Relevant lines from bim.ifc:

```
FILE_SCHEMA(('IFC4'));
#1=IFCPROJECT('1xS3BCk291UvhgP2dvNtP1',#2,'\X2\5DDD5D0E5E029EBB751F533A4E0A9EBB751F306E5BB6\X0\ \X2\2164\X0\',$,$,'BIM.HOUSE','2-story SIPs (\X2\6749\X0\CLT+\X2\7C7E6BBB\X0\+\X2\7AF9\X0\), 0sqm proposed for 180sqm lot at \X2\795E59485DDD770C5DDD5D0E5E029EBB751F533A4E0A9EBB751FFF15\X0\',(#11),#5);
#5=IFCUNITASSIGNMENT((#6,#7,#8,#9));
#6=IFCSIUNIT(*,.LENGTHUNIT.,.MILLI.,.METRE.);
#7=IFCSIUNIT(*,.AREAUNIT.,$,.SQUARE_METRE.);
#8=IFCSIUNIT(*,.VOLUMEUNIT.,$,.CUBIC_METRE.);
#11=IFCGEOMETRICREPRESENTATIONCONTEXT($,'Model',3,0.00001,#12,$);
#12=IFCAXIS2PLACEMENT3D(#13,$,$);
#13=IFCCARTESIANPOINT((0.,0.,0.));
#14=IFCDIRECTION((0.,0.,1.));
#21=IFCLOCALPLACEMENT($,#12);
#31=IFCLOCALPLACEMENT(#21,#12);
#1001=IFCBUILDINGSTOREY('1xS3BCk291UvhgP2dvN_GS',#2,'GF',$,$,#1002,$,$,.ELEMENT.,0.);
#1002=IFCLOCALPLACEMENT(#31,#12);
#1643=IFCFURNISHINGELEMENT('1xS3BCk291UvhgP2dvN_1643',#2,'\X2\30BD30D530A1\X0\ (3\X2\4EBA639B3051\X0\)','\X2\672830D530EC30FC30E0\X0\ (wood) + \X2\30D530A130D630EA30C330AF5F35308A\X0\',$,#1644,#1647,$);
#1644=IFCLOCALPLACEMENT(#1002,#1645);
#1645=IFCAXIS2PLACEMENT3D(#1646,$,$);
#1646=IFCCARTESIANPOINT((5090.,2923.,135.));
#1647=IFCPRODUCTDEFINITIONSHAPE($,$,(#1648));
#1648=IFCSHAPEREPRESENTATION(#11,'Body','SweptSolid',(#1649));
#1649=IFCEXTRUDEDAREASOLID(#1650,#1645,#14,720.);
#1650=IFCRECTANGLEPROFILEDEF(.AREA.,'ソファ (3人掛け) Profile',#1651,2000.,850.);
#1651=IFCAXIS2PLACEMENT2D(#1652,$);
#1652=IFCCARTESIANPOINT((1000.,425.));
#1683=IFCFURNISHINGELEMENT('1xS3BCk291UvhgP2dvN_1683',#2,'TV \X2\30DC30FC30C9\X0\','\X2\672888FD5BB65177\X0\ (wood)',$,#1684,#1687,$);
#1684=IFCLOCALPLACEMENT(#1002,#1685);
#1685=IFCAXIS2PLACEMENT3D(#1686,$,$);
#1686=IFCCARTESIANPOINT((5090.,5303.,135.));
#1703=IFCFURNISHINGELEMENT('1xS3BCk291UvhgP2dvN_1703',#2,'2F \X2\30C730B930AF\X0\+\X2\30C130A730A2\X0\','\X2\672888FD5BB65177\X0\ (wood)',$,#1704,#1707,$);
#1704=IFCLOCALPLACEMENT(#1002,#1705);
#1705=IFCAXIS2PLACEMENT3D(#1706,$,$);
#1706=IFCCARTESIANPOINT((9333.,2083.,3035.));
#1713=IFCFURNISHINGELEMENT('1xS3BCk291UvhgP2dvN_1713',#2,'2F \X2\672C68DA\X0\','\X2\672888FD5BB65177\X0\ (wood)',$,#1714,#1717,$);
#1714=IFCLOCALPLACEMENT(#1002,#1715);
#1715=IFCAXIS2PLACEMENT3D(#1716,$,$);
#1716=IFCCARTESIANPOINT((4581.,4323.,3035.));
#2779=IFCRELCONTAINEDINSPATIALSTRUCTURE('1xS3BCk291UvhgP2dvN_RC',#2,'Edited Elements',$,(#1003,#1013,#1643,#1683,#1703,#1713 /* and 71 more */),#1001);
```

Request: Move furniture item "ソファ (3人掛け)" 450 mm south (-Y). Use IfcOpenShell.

```python
import ifcopenshell
import ifcopenshell.api.geometry
import ifcopenshell.util.placement
import ifcopenshell.util.unit

model = ifcopenshell.open("bim.ifc")
unit_scale = ifcopenshell.util.unit.calculate_unit_scale(model)

item = model.by_guid("1xS3BCk291UvhgP2dvN_1643")
matrix = ifcopenshell.util.placement.get_local_placement(item.ObjectPlacement)
matrix[1, 3] -= 0.45 / unit_scale
ifcopenshell.api.geometry.edit_object_placement(model, product=item, matrix=matrix, is_si=False)

print(ifcopenshell.util.placement.get_local_placement(item.ObjectPlacement).round(3) + 0.0)

model.write("bim_v2.ifc")
```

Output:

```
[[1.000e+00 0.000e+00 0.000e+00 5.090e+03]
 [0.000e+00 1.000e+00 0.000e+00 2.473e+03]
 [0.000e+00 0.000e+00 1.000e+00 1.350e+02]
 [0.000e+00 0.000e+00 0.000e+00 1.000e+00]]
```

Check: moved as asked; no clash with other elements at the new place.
